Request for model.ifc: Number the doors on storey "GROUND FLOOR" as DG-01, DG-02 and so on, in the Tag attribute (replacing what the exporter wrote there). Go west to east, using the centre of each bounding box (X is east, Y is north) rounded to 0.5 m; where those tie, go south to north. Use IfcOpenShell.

First a look at what the model holds.

```python
import ifcopenshell
import ifcopenshell.util.element
import ifcopenshell.util.placement

model = ifcopenshell.open("model.ifc")
print(model.schema)
storey = next(s for s in model.by_type("IfcBuildingStorey") if s.Name == "GROUND FLOOR")
doors = [e for e in ifcopenshell.util.element.get_decomposition(storey) if e.is_a("IfcDoor")]
for e in sorted(doors, key=lambda e: e.id()):
    origin = ifcopenshell.util.placement.get_local_placement(e.ObjectPlacement)[:3, 3]
    print(e.id(), e.Tag, e.Name, origin.round(2) + 0.0, sep=" | ")
```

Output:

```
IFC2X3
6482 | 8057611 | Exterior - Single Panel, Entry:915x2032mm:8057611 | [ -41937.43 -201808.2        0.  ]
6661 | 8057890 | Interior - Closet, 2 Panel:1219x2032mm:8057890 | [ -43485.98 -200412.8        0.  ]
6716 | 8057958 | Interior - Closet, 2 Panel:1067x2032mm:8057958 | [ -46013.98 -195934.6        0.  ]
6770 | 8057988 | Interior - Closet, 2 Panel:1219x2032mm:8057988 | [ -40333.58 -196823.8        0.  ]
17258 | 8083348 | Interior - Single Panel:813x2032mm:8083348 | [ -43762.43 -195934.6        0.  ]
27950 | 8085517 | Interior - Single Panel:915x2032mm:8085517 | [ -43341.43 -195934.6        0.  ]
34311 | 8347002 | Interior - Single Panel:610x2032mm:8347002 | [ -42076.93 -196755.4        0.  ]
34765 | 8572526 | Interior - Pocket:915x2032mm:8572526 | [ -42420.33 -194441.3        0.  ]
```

```python
import ifcopenshell
import ifcopenshell.geom
import ifcopenshell.util.element
import ifcopenshell.util.shape

model = ifcopenshell.open("model.ifc")
settings = ifcopenshell.geom.settings()
settings.set("use-world-coords", True)


def centre(element):
    shape = ifcopenshell.geom.create_shape(settings, element)
    return ifcopenshell.util.shape.get_bbox_centroid(shape.geometry)


storey = next(s for s in model.by_type("IfcBuildingStorey") if s.Name == "GROUND FLOOR")
doors = [e for e in ifcopenshell.util.element.get_decomposition(storey) if e.is_a("IfcDoor")]

# Insertion points can sit at a corner or the storey origin, so sort by the geometry (in metres).
centres = {e: centre(e) for e in doors}
doors.sort(key=lambda e: (round(centres[e][0] / 0.5), centres[e][1]))

for i, e in enumerate(doors, start=1):
    number = f"DG-{i:02d}"
    e.Tag = number
    print(e.id(), number)

model.write("model_v2.ifc")
```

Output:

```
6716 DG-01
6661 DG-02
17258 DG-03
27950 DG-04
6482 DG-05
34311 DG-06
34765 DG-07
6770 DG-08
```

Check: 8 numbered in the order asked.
